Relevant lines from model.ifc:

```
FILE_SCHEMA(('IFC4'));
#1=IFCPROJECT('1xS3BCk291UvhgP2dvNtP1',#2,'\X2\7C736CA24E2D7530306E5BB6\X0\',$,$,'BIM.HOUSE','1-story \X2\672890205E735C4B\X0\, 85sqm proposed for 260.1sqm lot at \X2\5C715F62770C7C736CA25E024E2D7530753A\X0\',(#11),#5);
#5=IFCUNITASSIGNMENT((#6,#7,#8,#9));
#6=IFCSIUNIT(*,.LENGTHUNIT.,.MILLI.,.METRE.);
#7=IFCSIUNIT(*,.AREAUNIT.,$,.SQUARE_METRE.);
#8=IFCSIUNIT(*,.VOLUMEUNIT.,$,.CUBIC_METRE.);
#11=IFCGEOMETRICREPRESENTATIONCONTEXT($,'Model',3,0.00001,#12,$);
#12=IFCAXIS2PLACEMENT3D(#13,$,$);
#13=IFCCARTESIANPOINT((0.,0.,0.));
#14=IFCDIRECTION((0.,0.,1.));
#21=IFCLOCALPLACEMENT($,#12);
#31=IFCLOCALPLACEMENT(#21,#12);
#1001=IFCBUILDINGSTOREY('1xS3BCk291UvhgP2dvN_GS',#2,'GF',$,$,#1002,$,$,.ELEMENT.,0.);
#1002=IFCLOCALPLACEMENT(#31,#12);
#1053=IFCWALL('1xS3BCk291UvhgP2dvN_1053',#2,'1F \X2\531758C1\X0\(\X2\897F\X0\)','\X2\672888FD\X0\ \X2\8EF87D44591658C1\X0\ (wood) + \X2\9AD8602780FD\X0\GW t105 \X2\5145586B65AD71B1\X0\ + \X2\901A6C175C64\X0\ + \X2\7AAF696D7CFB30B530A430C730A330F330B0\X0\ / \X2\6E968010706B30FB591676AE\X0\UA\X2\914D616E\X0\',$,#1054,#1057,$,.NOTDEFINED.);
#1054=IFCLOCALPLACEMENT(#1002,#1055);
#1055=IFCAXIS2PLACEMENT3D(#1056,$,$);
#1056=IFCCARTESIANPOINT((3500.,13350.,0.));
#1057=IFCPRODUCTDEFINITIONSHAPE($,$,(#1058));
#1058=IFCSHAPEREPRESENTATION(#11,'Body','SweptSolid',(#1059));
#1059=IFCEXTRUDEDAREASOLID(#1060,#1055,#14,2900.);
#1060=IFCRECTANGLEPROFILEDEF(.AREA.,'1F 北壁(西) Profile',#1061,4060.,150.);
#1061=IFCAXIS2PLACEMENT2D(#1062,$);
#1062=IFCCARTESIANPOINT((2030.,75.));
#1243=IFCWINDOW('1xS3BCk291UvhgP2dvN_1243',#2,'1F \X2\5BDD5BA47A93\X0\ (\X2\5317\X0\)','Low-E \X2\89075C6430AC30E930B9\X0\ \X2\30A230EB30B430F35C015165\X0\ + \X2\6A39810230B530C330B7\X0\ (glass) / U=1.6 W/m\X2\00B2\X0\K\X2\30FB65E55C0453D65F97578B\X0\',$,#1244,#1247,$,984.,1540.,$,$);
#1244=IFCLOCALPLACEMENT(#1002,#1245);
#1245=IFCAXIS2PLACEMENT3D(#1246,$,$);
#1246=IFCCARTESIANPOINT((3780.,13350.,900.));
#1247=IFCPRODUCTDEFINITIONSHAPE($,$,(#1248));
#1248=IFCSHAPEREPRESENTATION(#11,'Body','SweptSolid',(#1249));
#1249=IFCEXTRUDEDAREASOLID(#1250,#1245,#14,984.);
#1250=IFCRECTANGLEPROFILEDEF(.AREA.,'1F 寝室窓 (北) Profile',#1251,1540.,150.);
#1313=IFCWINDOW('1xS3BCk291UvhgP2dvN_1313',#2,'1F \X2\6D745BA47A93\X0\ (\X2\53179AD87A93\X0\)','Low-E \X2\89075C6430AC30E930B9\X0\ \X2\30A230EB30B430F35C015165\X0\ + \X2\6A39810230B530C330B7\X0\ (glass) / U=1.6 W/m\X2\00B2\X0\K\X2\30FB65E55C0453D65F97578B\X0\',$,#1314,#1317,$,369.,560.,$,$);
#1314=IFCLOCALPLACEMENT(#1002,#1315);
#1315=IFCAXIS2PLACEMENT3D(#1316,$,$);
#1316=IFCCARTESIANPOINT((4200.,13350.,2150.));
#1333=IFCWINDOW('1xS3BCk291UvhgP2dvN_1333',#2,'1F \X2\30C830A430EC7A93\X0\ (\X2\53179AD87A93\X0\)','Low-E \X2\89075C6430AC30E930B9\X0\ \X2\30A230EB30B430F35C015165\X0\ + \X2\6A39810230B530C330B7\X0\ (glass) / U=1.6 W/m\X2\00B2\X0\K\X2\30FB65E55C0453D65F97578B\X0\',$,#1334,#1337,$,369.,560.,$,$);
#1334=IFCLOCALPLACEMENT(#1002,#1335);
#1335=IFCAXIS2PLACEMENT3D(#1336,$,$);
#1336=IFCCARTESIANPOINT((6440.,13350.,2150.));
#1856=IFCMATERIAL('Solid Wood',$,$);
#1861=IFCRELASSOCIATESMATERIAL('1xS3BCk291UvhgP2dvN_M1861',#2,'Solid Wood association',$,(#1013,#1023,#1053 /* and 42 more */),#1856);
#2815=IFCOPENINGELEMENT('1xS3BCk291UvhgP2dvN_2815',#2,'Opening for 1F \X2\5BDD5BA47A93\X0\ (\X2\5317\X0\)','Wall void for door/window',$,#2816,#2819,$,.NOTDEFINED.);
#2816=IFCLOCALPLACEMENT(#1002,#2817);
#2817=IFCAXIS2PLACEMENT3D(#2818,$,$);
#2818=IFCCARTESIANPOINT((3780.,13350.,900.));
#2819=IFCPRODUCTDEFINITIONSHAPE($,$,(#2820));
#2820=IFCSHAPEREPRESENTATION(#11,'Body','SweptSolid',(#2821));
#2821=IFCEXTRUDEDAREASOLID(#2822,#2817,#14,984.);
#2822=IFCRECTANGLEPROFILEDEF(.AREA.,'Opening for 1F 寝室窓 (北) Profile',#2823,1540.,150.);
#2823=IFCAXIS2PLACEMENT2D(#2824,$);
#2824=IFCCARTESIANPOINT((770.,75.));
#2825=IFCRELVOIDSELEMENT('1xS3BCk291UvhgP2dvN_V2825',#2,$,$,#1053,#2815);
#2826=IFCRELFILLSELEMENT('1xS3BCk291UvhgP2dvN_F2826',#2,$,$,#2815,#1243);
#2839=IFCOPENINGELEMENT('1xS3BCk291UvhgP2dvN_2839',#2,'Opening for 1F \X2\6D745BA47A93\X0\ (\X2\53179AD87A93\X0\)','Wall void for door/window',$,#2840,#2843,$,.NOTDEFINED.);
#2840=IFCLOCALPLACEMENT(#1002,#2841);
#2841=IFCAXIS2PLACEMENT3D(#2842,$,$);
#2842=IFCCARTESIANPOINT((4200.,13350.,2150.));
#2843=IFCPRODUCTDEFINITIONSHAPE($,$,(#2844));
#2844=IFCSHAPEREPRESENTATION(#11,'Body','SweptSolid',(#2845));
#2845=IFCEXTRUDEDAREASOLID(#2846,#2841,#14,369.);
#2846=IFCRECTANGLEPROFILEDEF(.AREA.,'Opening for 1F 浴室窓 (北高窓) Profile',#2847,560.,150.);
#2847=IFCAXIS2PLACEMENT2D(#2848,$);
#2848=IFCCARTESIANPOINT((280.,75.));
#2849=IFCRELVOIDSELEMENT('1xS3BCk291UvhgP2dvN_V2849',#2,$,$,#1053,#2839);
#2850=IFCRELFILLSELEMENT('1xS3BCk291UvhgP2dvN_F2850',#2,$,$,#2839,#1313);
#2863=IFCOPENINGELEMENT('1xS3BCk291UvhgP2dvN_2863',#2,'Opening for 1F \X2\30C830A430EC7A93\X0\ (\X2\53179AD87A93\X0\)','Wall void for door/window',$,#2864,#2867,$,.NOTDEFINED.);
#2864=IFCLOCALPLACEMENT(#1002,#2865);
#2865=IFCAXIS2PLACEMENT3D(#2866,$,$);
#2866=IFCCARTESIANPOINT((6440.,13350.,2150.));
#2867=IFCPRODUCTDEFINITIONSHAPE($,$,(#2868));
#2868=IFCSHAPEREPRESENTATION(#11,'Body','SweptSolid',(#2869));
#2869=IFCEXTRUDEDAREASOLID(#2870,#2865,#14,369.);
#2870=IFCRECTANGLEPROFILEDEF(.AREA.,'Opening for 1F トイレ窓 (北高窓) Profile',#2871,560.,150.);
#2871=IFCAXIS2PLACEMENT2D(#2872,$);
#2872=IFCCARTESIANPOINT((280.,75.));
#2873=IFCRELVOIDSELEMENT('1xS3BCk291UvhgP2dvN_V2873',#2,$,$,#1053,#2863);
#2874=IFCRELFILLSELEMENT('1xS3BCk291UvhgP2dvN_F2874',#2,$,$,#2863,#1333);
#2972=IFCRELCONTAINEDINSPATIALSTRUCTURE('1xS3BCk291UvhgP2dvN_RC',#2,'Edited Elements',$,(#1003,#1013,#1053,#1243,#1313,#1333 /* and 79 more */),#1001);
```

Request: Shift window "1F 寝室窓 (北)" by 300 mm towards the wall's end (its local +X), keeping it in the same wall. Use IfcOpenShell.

```python
import ifcopenshell
import ifcopenshell.api.geometry
import ifcopenshell.util.placement
import ifcopenshell.util.unit

model = ifcopenshell.open("model.ifc")
unit_scale = ifcopenshell.util.unit.calculate_unit_scale(model)

window = model.by_guid("1xS3BCk291UvhgP2dvN_1243")
opening = window.FillsVoids[0].RelatingOpeningElement
wall = opening.VoidsElements[0].RelatingBuildingElement

wall_matrix = ifcopenshell.util.placement.get_local_placement(wall.ObjectPlacement)
shift = wall_matrix[:3, 0] * 0.3 / unit_scale
before = ifcopenshell.util.placement.get_local_placement(window.ObjectPlacement)[:3, 3].copy()

# The window is not placed relative to its opening, so move both.
for product in (opening, window):
    matrix = ifcopenshell.util.placement.get_local_placement(product.ObjectPlacement)
    matrix[:3, 3] += shift
    ifcopenshell.api.geometry.edit_object_placement(model, product=product, matrix=matrix, is_si=False)

after = ifcopenshell.util.placement.get_local_placement(window.ObjectPlacement)[:3, 3]
print("window moved by", (after - before).round(3) + 0.0)

model.write("model-out.ifc")
```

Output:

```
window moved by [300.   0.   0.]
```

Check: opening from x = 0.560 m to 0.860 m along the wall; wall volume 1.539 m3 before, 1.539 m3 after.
